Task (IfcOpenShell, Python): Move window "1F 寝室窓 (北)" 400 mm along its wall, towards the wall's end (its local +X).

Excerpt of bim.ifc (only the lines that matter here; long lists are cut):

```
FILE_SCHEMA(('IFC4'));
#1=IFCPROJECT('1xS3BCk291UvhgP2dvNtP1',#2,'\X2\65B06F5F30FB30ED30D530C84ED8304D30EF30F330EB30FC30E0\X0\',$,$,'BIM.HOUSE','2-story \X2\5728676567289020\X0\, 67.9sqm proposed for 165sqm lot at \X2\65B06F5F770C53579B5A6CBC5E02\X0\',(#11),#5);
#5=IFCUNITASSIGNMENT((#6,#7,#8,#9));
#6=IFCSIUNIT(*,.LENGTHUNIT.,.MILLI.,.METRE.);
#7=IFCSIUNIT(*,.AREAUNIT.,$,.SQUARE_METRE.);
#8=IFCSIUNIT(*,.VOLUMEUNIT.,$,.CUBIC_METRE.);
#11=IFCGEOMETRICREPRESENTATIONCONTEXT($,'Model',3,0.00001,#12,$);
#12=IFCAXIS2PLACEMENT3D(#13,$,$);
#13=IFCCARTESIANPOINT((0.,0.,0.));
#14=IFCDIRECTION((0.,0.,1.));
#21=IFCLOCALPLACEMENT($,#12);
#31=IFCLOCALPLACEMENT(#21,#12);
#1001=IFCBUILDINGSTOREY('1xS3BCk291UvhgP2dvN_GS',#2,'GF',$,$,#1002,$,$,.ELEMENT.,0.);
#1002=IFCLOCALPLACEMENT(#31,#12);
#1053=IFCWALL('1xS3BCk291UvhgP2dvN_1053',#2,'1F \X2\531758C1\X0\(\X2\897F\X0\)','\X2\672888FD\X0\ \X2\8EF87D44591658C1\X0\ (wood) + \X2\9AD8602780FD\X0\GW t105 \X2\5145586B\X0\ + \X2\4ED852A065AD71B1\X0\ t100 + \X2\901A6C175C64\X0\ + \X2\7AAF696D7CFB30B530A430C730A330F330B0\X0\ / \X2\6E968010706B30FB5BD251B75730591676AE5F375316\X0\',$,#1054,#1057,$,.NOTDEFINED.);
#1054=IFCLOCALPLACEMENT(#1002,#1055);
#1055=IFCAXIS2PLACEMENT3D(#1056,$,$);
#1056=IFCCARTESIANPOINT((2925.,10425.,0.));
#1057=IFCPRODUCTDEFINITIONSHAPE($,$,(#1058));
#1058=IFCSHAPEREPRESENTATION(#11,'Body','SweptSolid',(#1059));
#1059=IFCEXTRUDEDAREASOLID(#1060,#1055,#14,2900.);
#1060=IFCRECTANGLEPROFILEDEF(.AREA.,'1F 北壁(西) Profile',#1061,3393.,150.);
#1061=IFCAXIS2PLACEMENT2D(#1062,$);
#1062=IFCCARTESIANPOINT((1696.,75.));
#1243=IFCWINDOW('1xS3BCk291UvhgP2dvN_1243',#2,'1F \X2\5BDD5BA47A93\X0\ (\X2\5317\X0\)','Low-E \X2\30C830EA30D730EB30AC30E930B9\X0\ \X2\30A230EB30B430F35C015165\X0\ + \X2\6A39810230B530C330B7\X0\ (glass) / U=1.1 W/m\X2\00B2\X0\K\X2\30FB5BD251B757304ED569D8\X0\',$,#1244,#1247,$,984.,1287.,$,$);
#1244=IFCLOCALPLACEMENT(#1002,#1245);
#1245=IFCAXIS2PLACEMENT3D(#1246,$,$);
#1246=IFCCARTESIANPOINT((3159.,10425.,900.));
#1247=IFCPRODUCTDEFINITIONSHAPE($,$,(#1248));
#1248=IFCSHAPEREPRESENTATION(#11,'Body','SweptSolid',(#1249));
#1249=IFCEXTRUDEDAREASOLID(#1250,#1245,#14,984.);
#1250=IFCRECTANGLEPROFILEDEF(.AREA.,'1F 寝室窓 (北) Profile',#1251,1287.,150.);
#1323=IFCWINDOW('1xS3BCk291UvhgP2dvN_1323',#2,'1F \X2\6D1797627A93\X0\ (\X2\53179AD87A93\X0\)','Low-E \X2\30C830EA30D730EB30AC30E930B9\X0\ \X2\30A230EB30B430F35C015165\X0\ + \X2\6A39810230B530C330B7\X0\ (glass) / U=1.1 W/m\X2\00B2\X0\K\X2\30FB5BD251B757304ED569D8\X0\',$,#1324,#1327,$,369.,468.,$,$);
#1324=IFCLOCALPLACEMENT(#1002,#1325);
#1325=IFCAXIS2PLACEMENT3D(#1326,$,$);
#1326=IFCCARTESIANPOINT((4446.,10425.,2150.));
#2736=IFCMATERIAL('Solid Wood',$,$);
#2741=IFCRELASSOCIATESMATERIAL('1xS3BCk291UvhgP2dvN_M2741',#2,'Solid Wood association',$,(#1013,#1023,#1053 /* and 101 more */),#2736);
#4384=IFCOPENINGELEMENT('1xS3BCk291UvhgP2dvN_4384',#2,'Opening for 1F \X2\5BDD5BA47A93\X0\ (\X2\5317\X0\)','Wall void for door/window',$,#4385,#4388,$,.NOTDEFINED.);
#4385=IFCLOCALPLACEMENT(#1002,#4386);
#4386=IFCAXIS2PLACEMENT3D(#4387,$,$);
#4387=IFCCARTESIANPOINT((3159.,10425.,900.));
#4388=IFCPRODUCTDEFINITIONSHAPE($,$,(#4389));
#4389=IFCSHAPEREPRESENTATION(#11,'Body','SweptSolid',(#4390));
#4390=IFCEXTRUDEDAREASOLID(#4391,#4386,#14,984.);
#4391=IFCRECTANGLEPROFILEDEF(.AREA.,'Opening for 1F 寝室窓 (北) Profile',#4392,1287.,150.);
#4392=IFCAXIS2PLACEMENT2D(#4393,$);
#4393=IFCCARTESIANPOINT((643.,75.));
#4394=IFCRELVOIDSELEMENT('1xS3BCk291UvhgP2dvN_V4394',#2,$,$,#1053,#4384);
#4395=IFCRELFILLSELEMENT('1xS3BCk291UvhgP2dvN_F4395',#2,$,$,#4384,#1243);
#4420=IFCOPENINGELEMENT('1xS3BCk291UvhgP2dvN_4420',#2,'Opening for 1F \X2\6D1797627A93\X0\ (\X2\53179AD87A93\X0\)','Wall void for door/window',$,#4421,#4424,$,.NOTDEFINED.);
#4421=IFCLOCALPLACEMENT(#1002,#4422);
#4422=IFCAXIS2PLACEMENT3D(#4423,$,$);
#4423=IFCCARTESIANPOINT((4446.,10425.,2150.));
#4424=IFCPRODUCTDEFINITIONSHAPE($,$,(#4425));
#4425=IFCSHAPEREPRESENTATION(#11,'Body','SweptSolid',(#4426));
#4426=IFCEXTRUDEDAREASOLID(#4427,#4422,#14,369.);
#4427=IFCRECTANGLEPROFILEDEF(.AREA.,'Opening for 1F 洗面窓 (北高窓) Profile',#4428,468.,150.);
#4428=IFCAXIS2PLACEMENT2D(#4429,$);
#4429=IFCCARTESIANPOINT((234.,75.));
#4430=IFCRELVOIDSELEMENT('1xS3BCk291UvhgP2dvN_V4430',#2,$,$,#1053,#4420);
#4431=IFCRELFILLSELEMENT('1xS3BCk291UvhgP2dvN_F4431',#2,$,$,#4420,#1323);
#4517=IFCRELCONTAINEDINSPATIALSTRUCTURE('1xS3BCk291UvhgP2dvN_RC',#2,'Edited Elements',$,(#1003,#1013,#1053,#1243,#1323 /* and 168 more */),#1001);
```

```python
import ifcopenshell
import ifcopenshell.api.geometry
import ifcopenshell.util.placement
import ifcopenshell.util.unit

model = ifcopenshell.open("bim.ifc")
unit_scale = ifcopenshell.util.unit.calculate_unit_scale(model)

window = model.by_guid("1xS3BCk291UvhgP2dvN_1243")
opening = window.FillsVoids[0].RelatingOpeningElement
wall = opening.VoidsElements[0].RelatingBuildingElement

wall_matrix = ifcopenshell.util.placement.get_local_placement(wall.ObjectPlacement)
shift = wall_matrix[:3, 0] * 0.4 / unit_scale
before = ifcopenshell.util.placement.get_local_placement(window.ObjectPlacement)[:3, 3].copy()

# The window is not placed relative to its opening, so move both.
for product in (opening, window):
    matrix = ifcopenshell.util.placement.get_local_placement(product.ObjectPlacement)
    matrix[:3, 3] += shift
    ifcopenshell.api.geometry.edit_object_placement(model, product=product, matrix=matrix, is_si=False)

after = ifcopenshell.util.placement.get_local_placement(window.ObjectPlacement)[:3, 3]
print("window moved by", (after - before).round(3) + 0.0)

model.write("bim_v2.ifc")
```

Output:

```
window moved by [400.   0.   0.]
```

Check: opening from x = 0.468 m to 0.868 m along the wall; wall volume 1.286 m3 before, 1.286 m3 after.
